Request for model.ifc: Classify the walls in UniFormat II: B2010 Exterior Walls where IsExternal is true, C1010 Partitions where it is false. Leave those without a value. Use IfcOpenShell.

First a look at what the model holds.

```python
import ifcopenshell
import ifcopenshell.util.element

model = ifcopenshell.open("model.ifc")
print(model.schema)
print("classifications:", [c.Name for c in model.by_type("IfcClassification")])
values = [ifcopenshell.util.element.get_pset(e, "Pset_WallCommon", "IsExternal") for e in model.by_type("IfcWall")]
for value in (True, False, None):
    print("IsExternal", value, values.count(value))
```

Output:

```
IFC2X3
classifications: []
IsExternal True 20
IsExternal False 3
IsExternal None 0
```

```python
import ifcopenshell
import ifcopenshell.api.classification
import ifcopenshell.util.element

model = ifcopenshell.open("model.ifc")

# IFC2X3 requires Source and Edition and has no link from the project to the system.
system = model.create_entity("IfcClassification", Source="ASTM", Edition="E1557", Name="UniFormat II")

walls = model.by_type("IfcWall")
external = {e: ifcopenshell.util.element.get_pset(e, "Pset_WallCommon", "IsExternal") for e in walls}
for flag, code, name in ((True, "B2010", "Exterior Walls"), (False, "C1010", "Partitions")):
    products = [e for e in walls if external[e] is flag]
    ifcopenshell.api.classification.add_reference(
        model, products=products, classification=system, identification=code, name=name
    )
    print(code, len(products))

model.write("model_edited.ifc")
```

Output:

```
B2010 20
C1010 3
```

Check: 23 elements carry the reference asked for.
